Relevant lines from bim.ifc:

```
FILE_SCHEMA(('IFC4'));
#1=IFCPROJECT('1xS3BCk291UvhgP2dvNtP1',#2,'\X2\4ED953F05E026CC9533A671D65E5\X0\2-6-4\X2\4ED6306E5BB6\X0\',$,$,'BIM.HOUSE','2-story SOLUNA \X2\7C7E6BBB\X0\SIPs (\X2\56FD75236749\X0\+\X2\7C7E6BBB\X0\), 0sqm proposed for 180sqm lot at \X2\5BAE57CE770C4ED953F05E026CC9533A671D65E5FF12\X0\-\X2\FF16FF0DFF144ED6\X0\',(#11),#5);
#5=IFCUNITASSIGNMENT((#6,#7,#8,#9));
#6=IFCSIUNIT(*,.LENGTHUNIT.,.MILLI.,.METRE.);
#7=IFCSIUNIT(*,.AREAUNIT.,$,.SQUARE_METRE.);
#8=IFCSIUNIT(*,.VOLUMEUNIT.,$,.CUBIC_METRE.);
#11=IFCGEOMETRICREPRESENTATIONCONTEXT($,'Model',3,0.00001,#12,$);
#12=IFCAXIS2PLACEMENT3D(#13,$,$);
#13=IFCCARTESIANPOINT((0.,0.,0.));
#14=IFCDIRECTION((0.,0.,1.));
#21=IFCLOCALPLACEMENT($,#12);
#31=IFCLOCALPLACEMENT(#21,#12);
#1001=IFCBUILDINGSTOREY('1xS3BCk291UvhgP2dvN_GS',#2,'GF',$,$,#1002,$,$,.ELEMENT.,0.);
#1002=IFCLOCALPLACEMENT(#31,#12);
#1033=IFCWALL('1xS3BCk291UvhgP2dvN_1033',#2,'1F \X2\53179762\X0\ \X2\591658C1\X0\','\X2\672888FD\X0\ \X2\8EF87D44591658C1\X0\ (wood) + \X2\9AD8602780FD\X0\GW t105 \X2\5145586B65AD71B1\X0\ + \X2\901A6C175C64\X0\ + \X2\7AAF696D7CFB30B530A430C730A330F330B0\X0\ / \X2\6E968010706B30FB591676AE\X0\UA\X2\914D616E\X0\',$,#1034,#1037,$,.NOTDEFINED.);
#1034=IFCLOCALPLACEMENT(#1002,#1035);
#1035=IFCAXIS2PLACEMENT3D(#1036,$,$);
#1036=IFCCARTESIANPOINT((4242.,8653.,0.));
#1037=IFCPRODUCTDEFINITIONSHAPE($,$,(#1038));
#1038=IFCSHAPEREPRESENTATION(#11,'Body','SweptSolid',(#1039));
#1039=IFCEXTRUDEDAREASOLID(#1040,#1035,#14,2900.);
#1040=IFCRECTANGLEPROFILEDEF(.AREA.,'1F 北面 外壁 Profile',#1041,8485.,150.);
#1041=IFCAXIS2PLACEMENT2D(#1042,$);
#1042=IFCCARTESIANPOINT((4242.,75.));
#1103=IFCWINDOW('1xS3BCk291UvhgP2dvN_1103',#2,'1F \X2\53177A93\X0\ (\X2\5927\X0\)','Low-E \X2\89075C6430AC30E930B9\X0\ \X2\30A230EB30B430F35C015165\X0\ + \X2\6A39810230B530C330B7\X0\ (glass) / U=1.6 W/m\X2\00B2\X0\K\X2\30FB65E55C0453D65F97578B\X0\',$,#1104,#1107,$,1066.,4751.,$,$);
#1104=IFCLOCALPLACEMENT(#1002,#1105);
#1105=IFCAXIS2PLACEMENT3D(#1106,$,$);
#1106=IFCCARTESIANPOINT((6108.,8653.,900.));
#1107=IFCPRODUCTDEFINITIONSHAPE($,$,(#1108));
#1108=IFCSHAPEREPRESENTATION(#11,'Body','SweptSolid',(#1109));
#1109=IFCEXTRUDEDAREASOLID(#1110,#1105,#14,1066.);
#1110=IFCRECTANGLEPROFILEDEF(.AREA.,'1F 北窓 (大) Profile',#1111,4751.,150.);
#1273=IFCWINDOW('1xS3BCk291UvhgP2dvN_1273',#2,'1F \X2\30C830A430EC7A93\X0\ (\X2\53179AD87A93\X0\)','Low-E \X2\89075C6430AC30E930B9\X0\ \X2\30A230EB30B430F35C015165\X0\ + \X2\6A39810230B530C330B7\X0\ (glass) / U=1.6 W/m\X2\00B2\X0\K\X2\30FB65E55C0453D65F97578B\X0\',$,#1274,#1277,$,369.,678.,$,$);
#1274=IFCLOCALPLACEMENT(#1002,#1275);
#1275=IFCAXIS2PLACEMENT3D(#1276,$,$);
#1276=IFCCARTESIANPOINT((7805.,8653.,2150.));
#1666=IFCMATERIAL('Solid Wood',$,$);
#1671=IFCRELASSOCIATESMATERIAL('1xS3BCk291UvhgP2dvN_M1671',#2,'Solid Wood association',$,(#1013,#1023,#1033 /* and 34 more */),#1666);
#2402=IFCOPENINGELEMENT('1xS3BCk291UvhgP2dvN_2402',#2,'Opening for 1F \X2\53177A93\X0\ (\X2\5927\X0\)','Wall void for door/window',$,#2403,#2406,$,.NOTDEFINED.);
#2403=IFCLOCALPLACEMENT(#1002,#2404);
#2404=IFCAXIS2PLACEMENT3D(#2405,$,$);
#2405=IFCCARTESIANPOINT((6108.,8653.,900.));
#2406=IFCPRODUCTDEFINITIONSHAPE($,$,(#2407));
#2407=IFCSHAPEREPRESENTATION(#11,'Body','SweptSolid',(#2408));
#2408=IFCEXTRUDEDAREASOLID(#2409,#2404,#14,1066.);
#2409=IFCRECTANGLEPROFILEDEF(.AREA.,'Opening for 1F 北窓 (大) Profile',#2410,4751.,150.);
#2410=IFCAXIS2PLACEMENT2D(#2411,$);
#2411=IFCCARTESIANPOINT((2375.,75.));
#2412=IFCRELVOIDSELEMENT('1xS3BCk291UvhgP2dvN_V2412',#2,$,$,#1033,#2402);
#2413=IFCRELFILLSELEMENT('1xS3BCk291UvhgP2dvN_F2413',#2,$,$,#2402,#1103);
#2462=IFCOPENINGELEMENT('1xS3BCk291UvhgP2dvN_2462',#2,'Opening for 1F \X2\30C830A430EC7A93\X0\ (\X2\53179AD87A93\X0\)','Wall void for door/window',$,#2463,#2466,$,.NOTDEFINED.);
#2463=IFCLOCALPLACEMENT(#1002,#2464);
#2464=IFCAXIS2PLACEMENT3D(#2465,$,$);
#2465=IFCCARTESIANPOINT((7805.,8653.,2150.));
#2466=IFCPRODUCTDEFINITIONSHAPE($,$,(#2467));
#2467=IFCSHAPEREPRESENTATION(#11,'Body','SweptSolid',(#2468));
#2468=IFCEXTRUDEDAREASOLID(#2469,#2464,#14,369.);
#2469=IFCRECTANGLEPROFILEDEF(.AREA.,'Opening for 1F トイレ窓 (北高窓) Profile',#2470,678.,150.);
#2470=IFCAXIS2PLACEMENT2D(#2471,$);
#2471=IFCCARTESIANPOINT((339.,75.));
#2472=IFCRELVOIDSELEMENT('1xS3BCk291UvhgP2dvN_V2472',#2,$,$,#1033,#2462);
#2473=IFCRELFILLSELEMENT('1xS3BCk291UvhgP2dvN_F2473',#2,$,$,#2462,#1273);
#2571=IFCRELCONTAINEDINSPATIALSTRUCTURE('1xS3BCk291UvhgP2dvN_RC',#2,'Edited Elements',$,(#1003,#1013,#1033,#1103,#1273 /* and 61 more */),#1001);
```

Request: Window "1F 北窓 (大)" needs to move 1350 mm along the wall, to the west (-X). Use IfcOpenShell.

```python
import ifcopenshell
import ifcopenshell.api.geometry
import ifcopenshell.util.placement
import ifcopenshell.util.unit

model = ifcopenshell.open("bim.ifc")
unit_scale = ifcopenshell.util.unit.calculate_unit_scale(model)

window = model.by_guid("1xS3BCk291UvhgP2dvN_1103")
opening = window.FillsVoids[0].RelatingOpeningElement
wall = opening.VoidsElements[0].RelatingBuildingElement

wall_matrix = ifcopenshell.util.placement.get_local_placement(wall.ObjectPlacement)
shift = wall_matrix[:3, 0] * -1.35 / unit_scale
before = ifcopenshell.util.placement.get_local_placement(window.ObjectPlacement)[:3, 3].copy()

# The window is not placed relative to its opening, so move both.
for product in (opening, window):
    matrix = ifcopenshell.util.placement.get_local_placement(product.ObjectPlacement)
    matrix[:3, 3] += shift
    ifcopenshell.api.geometry.edit_object_placement(model, product=product, matrix=matrix, is_si=False)

after = ifcopenshell.util.placement.get_local_placement(window.ObjectPlacement)[:3, 3]
print("window moved by", (after - before).round(3) + 0.0)

model.write("bim_edited.ifc")
```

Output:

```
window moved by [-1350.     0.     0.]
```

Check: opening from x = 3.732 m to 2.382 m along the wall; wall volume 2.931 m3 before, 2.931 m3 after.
